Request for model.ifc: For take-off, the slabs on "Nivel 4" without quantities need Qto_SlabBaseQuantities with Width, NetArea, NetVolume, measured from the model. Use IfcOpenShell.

First a look at what the model holds.

```python
import ifcopenshell
import ifcopenshell.util.element
import ifcopenshell.util.unit

model = ifcopenshell.open("model.ifc")
print(model.schema)
for unit_type in ("LENGTHUNIT", "AREAUNIT", "VOLUMEUNIT"):
    print(unit_type, ifcopenshell.util.unit.calculate_unit_scale(model, unit_type))
storey = next(s for s in model.by_type("IfcBuildingStorey") if s.Name == "Nivel 4")
slabs = [e for e in ifcopenshell.util.element.get_decomposition(storey) if e.is_a("IfcSlab")]
for e in sorted(slabs, key=lambda e: e.id()):
    print(e.id(), e.is_a(), e.Name, list(ifcopenshell.util.element.get_psets(e, qtos_only=True)), sep=" | ")
```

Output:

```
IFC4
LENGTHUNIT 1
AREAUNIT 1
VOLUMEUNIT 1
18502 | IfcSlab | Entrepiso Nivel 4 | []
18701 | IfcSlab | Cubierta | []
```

```python
import ifcopenshell
import ifcopenshell.api.pset
import ifcopenshell.geom
import ifcopenshell.util.element
import ifcopenshell.util.shape
import ifcopenshell.util.unit

model = ifcopenshell.open("model.ifc")
unit_scale = ifcopenshell.util.unit.calculate_unit_scale(model)
area_scale = ifcopenshell.util.unit.calculate_unit_scale(model, "AREAUNIT")
volume_scale = ifcopenshell.util.unit.calculate_unit_scale(model, "VOLUMEUNIT")
settings = ifcopenshell.geom.settings()

storey = next(s for s in model.by_type("IfcBuildingStorey") if s.Name == "Nivel 4")
slabs = [e for e in ifcopenshell.util.element.get_decomposition(storey) if e.is_a("IfcSlab")]

for e in sorted(slabs, key=lambda e: e.id()):
    if ifcopenshell.util.element.get_psets(e, qtos_only=True, should_inherit=False):
        continue
    # Geometry comes back in metres, in the element's own axes.
    shape = ifcopenshell.geom.create_shape(settings, e)
    values = {
        "Width": ifcopenshell.util.shape.get_z(shape.geometry) / unit_scale,
        "NetArea": ifcopenshell.util.shape.get_footprint_area(shape.geometry) / area_scale,
        "NetVolume": ifcopenshell.util.shape.get_volume(shape.geometry) / volume_scale,
    }
    qto = ifcopenshell.api.pset.add_qto(model, product=e, name="Qto_SlabBaseQuantities")
    ifcopenshell.api.pset.edit_qto(model, qto=qto, properties=values)
    print(e.id(), {k: round(v, 3) for k, v in values.items()})

model.write("model_v2.ifc")
```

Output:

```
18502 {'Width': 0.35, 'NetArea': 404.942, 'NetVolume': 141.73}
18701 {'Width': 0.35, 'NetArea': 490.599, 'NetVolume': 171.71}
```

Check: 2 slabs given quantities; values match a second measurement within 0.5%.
